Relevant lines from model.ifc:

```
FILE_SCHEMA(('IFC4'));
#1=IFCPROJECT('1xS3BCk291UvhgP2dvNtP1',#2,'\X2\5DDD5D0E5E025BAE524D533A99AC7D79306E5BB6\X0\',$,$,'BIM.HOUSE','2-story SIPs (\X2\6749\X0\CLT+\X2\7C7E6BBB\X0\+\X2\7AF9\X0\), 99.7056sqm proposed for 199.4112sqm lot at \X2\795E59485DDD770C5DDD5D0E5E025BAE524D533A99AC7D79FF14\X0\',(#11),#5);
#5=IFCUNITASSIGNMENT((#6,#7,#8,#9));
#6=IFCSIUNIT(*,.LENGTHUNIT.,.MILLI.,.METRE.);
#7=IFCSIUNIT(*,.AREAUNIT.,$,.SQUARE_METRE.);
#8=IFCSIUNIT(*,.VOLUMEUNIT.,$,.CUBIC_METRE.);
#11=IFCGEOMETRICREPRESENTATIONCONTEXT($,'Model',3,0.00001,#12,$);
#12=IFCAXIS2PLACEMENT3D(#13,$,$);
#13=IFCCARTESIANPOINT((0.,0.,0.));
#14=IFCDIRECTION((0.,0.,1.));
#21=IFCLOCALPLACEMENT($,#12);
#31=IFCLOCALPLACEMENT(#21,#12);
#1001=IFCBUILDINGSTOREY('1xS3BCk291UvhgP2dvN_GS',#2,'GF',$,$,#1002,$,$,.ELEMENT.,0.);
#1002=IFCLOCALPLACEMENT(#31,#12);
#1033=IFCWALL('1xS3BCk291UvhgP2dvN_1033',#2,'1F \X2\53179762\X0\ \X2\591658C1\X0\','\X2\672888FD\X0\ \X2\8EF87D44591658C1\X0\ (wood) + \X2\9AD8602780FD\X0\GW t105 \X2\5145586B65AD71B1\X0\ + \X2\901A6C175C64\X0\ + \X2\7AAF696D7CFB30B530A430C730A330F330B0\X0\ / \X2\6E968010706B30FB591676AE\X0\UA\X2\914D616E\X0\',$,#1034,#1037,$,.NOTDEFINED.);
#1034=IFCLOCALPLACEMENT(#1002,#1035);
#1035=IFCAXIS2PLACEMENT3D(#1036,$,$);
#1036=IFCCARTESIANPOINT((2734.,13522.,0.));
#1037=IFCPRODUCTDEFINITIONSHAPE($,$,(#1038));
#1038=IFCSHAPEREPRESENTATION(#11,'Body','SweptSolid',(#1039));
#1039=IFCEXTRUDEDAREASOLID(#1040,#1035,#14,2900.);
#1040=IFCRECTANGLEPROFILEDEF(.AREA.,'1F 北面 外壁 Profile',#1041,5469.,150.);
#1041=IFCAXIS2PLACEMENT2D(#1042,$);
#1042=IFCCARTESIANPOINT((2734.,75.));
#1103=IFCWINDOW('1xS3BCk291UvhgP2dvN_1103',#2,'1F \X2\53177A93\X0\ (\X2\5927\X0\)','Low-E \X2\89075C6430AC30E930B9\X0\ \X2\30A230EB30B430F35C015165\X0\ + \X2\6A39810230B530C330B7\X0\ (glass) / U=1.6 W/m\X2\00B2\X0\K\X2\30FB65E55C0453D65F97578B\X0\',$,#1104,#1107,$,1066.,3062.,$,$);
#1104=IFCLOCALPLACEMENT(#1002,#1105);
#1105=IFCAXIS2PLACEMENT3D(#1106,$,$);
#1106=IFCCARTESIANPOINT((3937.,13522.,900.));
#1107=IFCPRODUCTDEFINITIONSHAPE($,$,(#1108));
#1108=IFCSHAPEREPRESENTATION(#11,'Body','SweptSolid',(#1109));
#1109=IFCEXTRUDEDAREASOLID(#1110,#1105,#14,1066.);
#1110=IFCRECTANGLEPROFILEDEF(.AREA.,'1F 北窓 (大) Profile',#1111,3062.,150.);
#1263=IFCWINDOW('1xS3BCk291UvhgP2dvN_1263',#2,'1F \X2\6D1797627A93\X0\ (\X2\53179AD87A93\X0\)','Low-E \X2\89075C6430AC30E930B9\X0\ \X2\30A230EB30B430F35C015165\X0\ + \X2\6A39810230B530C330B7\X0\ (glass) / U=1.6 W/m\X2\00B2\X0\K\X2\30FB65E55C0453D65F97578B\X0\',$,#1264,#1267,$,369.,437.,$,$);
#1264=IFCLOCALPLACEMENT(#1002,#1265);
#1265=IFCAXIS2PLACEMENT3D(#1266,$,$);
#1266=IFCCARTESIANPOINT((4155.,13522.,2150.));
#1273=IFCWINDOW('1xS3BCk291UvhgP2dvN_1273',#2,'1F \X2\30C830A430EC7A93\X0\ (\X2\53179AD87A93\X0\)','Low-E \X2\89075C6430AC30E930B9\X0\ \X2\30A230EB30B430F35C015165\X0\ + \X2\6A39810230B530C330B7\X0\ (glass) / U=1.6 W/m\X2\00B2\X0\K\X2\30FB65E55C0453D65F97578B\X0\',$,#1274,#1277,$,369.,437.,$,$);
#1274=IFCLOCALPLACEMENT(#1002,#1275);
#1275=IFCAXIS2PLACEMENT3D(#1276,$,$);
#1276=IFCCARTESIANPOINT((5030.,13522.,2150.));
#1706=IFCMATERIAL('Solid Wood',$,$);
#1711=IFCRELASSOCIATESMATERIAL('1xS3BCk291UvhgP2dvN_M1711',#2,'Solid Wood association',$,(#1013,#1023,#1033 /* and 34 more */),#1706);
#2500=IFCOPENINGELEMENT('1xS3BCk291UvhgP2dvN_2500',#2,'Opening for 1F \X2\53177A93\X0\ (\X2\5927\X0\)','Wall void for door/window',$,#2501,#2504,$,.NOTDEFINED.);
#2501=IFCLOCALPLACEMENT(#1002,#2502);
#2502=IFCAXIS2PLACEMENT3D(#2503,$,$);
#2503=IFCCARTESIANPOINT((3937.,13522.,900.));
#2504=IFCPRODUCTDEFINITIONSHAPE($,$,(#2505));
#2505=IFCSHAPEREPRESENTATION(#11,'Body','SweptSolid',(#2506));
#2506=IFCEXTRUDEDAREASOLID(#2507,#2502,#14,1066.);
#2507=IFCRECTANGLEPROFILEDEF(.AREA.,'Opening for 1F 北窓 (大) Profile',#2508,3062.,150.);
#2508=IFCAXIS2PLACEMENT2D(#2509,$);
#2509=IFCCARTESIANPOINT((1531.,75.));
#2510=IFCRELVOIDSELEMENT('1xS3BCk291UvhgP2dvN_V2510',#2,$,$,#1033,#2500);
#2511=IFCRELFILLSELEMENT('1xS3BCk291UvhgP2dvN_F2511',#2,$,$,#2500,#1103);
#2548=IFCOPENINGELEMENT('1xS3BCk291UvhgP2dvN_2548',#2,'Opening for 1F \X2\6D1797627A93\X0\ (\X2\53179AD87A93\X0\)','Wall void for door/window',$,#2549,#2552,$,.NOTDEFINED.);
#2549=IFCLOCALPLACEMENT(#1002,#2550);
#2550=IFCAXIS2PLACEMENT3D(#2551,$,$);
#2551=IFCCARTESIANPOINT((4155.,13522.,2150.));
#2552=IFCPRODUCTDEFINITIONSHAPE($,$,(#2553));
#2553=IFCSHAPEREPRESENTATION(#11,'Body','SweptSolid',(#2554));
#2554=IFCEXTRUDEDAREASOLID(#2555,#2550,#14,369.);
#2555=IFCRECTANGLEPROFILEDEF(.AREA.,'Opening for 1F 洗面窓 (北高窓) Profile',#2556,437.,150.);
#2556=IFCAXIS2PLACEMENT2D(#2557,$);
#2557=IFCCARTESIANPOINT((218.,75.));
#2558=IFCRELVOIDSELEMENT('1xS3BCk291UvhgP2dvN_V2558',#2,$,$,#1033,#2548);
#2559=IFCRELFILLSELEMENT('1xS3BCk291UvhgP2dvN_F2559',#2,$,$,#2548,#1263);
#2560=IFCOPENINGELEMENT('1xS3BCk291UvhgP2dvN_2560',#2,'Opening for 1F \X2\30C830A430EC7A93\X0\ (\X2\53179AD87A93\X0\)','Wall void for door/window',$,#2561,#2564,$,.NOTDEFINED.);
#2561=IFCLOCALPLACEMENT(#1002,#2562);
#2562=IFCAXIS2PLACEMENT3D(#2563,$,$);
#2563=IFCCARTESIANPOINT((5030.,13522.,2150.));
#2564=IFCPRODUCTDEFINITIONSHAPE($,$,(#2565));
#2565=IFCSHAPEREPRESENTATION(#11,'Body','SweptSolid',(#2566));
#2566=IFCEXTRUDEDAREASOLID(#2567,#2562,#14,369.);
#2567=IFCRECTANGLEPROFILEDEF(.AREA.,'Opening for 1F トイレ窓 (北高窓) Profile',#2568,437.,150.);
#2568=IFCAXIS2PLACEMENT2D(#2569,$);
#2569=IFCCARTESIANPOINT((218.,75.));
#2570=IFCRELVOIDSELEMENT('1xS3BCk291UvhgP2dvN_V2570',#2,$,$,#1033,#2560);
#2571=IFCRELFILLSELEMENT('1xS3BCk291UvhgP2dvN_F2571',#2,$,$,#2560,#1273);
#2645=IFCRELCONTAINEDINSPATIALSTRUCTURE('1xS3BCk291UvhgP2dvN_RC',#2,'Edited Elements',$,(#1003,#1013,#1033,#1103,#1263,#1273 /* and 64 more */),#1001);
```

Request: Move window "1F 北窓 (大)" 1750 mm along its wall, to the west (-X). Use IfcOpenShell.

```python
import ifcopenshell
import ifcopenshell.api.geometry
import ifcopenshell.util.placement
import ifcopenshell.util.unit

model = ifcopenshell.open("model.ifc")
unit_scale = ifcopenshell.util.unit.calculate_unit_scale(model)

window = model.by_guid("1xS3BCk291UvhgP2dvN_1103")
opening = window.FillsVoids[0].RelatingOpeningElement
wall = opening.VoidsElements[0].RelatingBuildingElement

wall_matrix = ifcopenshell.util.placement.get_local_placement(wall.ObjectPlacement)
shift = wall_matrix[:3, 0] * -1.75 / unit_scale
before = ifcopenshell.util.placement.get_local_placement(window.ObjectPlacement)[:3, 3].copy()

# The window is not placed relative to its opening, so move both.
for product in (opening, window):
    matrix = ifcopenshell.util.placement.get_local_placement(product.ObjectPlacement)
    matrix[:3, 3] += shift
    ifcopenshell.api.geometry.edit_object_placement(model, product=product, matrix=matrix, is_si=False)

after = ifcopenshell.util.placement.get_local_placement(window.ObjectPlacement)[:3, 3]
print("window moved by", (after - before).round(3) + 0.0)

model.write("model_v2.ifc")
```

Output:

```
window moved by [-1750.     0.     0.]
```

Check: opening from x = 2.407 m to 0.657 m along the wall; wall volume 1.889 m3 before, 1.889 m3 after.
